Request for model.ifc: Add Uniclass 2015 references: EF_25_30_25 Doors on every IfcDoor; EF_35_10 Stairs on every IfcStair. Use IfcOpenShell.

First a look at what the model holds.

```python
import ifcopenshell

model = ifcopenshell.open("model.ifc")
print(model.schema)
print("classifications:", [c.Name for c in model.by_type("IfcClassification")])
for ifc_class in ("IfcDoor", "IfcRoof", "IfcStair", "IfcWall", "IfcWindow"):
    print(ifc_class, len(model.by_type(ifc_class)))
```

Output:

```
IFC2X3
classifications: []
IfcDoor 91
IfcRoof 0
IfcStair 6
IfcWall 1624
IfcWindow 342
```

```python
import ifcopenshell
import ifcopenshell.api.classification

model = ifcopenshell.open("model.ifc")

# IFC2X3 requires Source and Edition and has no link from the project to the system.
system = model.create_entity("IfcClassification", Source="NBS", Edition="2015", Name="Uniclass 2015")

codes = {
    "IfcDoor": ("EF_25_30_25", "Doors"),
    "IfcStair": ("EF_35_10", "Stairs"),
}
for ifc_class, (code, name) in codes.items():
    products = model.by_type(ifc_class)
    ifcopenshell.api.classification.add_reference(
        model, products=products, classification=system, identification=code, name=name
    )
    print(code, len(products))

model.write("model_edited.ifc")
```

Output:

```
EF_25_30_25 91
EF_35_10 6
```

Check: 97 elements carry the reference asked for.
